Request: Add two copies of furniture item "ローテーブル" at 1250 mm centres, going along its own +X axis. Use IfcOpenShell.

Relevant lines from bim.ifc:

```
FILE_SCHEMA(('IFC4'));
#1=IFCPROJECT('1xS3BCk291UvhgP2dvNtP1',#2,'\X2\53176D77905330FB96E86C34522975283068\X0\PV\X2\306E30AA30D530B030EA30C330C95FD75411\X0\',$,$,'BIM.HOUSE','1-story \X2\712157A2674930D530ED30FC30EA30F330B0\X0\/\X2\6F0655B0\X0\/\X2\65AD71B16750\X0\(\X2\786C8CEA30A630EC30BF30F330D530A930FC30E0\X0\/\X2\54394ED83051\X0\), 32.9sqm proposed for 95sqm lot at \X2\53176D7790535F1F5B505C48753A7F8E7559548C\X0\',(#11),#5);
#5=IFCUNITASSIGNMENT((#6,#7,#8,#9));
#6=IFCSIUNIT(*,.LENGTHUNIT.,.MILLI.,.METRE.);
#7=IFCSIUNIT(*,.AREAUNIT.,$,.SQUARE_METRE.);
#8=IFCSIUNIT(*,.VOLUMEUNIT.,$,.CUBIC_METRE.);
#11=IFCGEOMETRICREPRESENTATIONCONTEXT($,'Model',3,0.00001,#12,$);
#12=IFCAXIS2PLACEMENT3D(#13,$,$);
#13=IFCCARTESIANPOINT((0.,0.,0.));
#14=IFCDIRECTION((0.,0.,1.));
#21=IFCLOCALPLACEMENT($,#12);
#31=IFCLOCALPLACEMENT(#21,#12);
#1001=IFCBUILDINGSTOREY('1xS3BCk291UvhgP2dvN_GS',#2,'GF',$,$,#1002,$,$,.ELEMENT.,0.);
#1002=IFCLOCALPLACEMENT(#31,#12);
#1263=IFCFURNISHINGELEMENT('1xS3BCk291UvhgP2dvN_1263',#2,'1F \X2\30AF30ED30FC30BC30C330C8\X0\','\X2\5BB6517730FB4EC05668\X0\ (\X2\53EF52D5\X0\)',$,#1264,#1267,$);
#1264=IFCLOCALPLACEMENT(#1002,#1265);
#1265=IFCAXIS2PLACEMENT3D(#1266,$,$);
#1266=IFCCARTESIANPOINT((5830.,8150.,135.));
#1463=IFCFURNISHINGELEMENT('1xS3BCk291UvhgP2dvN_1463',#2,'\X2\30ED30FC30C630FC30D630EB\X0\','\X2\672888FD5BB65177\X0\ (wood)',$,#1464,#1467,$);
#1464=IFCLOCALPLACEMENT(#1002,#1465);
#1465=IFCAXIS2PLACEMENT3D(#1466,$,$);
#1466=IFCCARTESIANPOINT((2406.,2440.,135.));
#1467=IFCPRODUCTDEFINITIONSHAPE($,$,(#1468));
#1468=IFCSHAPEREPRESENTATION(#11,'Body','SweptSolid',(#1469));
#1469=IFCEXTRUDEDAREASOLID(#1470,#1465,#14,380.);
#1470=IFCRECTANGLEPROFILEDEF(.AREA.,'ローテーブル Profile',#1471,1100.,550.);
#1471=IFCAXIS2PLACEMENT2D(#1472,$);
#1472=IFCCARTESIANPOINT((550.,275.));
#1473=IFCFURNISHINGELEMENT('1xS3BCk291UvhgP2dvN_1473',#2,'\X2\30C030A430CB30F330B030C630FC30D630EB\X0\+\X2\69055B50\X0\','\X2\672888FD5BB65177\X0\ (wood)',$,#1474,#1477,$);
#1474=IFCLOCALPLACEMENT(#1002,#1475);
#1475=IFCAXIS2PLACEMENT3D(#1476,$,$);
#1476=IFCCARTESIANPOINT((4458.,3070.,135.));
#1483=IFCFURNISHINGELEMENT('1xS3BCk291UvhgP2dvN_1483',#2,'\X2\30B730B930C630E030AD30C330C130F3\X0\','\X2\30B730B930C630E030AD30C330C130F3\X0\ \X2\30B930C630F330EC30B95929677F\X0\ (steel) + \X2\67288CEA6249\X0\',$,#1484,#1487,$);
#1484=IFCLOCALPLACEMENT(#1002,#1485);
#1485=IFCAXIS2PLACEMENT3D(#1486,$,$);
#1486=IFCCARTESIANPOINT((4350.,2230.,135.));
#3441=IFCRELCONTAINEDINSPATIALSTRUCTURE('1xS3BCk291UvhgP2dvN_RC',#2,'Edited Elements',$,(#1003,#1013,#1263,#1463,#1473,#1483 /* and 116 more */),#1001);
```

```python
import ifcopenshell
import ifcopenshell.api.geometry
import ifcopenshell.api.root
import ifcopenshell.util.element
import ifcopenshell.util.placement
import ifcopenshell.util.unit

model = ifcopenshell.open("bim.ifc")
unit_scale = ifcopenshell.util.unit.calculate_unit_scale(model)


def reuse_history(source, copy):
    """copy_class also copies each property set's owner history, people and application; keep the originals."""
    for rel in copy.IsDefinedBy:
        if rel.is_a("IfcRelDefinesByProperties") and (history := rel.RelatingPropertyDefinition.OwnerHistory):
            rel.RelatingPropertyDefinition.OwnerHistory = source.OwnerHistory
            ifcopenshell.util.element.remove_deep2(model, history)


source = model.by_id(1463)
base = ifcopenshell.util.placement.get_local_placement(source.ObjectPlacement)
step = base[:3, 0] * 1.25 / unit_scale

for i in range(1, 3):
    copy = ifcopenshell.api.root.copy_class(model, product=source)
    copy.Representation = ifcopenshell.util.element.copy_deep(
        model, source.Representation, exclude=["IfcGeometricRepresentationContext", "IfcRepresentationMap"]
    )
    reuse_history(source, copy)
    matrix = base.copy()
    matrix[:3, 3] += i * step
    print("added at", matrix[:3, 3].round(3) + 0.0)
    ifcopenshell.api.geometry.edit_object_placement(model, product=copy, matrix=matrix, is_si=False)

model.write("bim_rev.ifc")
```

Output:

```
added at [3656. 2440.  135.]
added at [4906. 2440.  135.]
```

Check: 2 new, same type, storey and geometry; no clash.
